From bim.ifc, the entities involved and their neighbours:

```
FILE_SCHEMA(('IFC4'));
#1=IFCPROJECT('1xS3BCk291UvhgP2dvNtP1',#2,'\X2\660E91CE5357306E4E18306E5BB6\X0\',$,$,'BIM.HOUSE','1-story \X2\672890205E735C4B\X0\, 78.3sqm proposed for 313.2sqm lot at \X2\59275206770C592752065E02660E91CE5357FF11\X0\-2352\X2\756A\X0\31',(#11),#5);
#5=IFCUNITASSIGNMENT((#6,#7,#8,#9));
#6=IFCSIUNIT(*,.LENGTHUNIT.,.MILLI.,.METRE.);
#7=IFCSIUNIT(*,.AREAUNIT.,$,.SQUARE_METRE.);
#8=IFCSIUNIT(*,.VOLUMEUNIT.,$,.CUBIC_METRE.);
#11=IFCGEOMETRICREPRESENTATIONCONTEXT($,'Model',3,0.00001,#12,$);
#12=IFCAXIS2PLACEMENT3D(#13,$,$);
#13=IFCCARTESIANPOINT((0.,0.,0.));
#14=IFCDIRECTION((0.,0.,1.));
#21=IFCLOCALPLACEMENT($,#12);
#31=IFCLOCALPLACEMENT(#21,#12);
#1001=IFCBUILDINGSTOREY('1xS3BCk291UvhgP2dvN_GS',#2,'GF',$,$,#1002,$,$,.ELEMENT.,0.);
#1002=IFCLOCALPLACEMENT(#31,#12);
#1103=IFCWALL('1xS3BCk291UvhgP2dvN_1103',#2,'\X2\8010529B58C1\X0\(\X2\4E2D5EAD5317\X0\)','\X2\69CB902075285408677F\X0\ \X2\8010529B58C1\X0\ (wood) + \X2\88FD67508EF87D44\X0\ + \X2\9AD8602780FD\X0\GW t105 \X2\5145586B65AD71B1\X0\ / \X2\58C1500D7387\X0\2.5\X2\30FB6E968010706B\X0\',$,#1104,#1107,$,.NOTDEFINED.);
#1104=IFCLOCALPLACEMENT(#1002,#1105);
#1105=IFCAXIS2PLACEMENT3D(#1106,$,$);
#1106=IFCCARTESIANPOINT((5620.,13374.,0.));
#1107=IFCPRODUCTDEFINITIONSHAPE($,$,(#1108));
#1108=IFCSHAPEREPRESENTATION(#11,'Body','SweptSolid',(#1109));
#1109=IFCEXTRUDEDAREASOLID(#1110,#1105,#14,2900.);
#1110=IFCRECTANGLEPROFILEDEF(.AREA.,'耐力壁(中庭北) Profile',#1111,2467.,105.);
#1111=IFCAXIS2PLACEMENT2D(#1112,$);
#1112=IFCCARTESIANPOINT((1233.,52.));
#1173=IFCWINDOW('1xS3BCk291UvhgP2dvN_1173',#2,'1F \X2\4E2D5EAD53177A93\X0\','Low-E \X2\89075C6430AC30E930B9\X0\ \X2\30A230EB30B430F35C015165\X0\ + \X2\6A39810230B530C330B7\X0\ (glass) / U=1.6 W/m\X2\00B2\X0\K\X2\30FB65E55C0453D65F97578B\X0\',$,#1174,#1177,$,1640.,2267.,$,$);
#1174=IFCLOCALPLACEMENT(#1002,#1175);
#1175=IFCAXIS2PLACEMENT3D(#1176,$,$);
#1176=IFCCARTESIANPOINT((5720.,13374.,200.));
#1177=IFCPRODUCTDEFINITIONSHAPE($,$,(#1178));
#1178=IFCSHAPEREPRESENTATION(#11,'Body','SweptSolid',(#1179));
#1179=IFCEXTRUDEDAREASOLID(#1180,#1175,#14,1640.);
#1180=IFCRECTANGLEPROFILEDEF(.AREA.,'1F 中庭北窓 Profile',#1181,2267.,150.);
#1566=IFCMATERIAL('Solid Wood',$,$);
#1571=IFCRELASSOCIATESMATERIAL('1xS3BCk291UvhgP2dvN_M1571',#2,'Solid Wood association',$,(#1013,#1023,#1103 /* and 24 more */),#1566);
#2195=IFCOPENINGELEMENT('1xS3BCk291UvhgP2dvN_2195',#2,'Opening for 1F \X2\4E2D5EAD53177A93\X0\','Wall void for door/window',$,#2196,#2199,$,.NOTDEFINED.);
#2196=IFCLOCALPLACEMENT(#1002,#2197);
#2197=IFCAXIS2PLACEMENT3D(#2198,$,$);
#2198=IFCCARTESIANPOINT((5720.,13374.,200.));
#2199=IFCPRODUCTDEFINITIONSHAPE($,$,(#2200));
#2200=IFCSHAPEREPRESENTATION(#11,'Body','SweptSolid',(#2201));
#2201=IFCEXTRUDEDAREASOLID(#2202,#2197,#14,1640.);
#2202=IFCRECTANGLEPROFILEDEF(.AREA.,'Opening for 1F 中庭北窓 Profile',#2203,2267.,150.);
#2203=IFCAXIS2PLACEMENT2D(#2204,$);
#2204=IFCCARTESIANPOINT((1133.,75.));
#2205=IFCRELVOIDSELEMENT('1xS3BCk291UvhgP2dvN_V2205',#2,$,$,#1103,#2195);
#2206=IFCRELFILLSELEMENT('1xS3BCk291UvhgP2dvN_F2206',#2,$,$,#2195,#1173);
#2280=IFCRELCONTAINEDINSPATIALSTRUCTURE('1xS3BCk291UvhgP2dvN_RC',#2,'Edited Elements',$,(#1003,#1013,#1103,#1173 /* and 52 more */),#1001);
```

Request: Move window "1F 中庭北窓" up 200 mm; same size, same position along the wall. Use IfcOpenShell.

```python
import numpy as np
import ifcopenshell
import ifcopenshell.api.geometry
import ifcopenshell.util.placement
import ifcopenshell.util.unit

model = ifcopenshell.open("bim.ifc")
unit_scale = ifcopenshell.util.unit.calculate_unit_scale(model)

window = model.by_id(1173)
opening = window.FillsVoids[0].RelatingOpeningElement
dz = 0.2 / unit_scale

shift = np.array([0.0, 0.0, dz])
# The window is not placed relative to its opening, so move both.
for product in (opening, window):
    matrix = ifcopenshell.util.placement.get_local_placement(product.ObjectPlacement)
    matrix[:3, 3] += shift
    ifcopenshell.api.geometry.edit_object_placement(model, product=product, matrix=matrix, is_si=False)

print(f"moved by {dz * unit_scale:+.3f} m")

model.write("bim_rev.ifc")
```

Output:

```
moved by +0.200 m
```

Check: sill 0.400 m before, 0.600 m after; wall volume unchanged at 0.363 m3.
